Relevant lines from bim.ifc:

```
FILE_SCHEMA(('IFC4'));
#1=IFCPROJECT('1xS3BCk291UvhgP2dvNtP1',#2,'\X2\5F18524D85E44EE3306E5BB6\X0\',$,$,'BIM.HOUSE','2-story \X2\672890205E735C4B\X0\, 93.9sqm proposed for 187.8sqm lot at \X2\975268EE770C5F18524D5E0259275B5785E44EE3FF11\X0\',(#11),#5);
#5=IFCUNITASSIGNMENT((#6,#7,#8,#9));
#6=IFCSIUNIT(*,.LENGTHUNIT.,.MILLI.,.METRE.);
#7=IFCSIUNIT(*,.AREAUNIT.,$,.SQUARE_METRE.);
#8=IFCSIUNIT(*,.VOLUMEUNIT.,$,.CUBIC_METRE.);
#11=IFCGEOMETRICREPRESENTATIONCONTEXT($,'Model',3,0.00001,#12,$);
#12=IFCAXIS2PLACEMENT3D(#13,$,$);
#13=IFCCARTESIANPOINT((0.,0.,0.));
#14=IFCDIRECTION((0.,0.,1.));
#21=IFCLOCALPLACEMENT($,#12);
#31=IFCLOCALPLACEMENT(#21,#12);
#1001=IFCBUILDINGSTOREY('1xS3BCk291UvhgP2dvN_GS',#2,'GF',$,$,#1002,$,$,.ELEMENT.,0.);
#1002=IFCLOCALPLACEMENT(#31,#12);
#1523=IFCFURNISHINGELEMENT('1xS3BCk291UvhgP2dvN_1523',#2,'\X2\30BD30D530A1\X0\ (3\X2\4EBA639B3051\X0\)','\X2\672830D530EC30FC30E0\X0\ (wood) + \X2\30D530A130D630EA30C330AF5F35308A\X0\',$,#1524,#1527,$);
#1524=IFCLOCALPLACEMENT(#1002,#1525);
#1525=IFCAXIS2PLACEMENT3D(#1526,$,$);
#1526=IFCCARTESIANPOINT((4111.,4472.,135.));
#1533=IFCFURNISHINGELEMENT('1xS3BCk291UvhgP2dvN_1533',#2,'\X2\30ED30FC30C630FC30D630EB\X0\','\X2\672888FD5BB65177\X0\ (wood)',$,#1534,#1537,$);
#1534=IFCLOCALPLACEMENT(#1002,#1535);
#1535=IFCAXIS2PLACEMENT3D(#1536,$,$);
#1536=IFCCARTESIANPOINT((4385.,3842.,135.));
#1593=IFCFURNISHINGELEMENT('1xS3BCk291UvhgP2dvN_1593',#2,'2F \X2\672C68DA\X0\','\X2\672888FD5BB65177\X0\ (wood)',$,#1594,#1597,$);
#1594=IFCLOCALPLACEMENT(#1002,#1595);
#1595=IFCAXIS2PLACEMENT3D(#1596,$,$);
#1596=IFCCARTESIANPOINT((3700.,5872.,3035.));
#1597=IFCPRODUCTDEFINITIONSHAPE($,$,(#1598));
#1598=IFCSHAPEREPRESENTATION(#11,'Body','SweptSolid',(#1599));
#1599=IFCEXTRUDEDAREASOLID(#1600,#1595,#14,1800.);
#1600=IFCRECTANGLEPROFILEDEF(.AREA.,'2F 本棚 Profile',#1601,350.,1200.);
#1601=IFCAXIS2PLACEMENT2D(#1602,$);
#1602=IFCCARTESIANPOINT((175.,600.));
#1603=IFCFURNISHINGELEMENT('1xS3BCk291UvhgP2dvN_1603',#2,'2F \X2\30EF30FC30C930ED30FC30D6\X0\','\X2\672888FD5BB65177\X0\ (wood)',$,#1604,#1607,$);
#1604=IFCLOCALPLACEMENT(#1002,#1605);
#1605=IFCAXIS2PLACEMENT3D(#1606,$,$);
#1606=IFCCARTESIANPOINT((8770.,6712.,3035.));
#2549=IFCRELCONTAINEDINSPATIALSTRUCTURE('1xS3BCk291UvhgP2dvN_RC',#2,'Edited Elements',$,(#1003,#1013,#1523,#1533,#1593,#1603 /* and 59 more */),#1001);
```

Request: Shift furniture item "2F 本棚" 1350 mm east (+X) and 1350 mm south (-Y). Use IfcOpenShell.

```python
import ifcopenshell
import ifcopenshell.api.geometry
import ifcopenshell.util.placement
import ifcopenshell.util.unit

model = ifcopenshell.open("bim.ifc")
unit_scale = ifcopenshell.util.unit.calculate_unit_scale(model)

item = model.by_id(1593)
matrix = ifcopenshell.util.placement.get_local_placement(item.ObjectPlacement)
matrix[0, 3] += 1.35 / unit_scale
matrix[1, 3] -= 1.35 / unit_scale
ifcopenshell.api.geometry.edit_object_placement(model, product=item, matrix=matrix, is_si=False)

print(ifcopenshell.util.placement.get_local_placement(item.ObjectPlacement).round(3) + 0.0)

model.write("bim_rev.ifc")
```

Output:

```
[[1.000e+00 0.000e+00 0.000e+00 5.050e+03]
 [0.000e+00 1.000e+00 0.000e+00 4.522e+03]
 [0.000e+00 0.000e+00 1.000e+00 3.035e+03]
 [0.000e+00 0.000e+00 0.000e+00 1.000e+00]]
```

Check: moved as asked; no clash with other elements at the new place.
